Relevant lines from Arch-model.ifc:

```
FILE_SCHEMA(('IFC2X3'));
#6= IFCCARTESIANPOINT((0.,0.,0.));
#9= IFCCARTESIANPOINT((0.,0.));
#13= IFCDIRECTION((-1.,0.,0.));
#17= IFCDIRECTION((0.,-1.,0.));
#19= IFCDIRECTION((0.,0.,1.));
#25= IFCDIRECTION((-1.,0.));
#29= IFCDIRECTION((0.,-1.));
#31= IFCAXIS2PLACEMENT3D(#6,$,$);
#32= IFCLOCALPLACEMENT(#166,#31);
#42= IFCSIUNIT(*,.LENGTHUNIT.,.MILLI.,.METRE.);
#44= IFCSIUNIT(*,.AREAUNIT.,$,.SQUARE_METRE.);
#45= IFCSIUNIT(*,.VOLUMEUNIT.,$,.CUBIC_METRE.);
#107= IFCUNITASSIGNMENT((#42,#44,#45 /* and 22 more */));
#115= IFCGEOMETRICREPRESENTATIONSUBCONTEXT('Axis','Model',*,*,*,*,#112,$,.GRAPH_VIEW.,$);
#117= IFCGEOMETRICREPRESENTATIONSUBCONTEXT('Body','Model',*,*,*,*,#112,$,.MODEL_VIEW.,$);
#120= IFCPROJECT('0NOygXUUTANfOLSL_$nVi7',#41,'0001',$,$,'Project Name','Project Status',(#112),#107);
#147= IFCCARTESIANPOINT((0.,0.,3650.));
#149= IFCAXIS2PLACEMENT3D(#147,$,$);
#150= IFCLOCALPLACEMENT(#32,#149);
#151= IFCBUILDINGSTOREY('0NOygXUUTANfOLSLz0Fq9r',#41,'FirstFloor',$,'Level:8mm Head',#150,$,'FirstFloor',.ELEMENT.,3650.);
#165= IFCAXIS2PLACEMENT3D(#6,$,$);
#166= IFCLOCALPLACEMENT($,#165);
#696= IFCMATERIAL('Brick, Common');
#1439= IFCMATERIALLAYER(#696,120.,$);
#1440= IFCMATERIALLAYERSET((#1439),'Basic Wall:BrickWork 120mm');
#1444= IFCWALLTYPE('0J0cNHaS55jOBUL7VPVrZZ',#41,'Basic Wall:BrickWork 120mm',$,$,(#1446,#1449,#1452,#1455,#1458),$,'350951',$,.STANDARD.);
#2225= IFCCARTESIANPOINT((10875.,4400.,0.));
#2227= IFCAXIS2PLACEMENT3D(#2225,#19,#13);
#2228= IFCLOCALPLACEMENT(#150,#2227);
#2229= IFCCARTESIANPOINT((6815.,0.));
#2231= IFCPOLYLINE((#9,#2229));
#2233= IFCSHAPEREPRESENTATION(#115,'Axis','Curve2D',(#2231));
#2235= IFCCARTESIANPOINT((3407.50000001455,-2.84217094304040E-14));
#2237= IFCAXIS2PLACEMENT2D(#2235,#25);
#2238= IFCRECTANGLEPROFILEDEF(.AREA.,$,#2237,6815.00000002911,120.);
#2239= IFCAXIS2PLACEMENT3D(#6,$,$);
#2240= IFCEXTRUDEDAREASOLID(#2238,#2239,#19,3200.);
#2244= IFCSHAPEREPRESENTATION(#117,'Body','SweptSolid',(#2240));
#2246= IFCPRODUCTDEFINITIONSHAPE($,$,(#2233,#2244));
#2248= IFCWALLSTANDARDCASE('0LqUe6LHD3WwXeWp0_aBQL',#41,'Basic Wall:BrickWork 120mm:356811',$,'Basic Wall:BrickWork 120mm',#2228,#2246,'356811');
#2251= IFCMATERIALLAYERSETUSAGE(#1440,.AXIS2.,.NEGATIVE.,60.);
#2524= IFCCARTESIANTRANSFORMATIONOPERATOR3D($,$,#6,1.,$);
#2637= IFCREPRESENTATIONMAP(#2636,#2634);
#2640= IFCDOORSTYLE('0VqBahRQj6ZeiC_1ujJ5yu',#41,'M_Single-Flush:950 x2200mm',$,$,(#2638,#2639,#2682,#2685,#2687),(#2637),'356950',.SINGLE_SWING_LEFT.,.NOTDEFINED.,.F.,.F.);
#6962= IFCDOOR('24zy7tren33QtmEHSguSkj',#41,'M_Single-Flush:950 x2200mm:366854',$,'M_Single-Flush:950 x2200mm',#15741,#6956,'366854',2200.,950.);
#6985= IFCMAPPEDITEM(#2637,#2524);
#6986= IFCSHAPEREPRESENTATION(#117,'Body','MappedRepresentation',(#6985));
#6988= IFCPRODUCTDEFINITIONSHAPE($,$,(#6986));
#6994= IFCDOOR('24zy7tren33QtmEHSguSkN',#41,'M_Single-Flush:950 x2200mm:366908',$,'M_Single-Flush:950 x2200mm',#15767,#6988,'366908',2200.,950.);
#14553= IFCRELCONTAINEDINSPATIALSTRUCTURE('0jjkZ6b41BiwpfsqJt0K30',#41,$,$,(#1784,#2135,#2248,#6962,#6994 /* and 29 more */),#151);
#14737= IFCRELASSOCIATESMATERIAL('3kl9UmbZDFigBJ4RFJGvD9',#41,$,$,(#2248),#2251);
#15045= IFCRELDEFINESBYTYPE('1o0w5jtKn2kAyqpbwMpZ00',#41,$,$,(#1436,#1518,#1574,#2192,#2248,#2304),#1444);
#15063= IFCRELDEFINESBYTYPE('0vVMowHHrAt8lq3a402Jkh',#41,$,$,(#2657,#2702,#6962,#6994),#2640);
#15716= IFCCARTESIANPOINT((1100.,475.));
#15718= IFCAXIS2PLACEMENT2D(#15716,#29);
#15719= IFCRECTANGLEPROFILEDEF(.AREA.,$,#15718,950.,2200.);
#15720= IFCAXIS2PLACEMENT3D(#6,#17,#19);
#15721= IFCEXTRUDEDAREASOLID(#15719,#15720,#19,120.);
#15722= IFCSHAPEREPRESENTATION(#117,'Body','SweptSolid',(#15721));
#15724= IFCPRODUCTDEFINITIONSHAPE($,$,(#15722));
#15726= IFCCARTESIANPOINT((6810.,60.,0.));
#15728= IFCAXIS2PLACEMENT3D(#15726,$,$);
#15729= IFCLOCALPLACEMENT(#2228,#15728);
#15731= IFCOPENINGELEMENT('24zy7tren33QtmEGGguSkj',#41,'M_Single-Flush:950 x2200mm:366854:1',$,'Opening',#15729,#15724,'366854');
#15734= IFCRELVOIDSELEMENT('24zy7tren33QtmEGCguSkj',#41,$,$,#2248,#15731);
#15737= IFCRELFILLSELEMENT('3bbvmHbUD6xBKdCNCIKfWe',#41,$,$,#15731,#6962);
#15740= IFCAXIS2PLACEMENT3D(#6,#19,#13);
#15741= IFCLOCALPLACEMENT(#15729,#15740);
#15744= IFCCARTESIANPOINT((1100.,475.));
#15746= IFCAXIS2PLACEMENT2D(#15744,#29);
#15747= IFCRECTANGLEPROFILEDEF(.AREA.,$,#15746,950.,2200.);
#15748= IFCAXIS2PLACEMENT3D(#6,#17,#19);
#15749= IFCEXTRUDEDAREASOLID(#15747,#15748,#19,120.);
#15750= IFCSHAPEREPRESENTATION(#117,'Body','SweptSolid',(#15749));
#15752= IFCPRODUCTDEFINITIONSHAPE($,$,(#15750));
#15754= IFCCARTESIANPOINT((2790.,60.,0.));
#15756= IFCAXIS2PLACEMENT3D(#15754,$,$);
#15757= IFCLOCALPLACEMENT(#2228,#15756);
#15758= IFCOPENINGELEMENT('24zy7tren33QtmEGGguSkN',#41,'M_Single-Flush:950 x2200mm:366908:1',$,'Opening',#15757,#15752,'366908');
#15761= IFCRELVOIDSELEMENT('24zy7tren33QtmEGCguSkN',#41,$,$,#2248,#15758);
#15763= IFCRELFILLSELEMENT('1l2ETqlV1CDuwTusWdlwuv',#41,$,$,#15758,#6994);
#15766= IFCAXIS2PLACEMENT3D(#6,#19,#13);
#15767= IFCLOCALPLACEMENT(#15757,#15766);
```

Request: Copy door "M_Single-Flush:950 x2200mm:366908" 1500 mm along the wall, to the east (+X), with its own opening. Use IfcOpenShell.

```python
import ifcopenshell
import ifcopenshell.api.feature
import ifcopenshell.api.geometry
import ifcopenshell.api.root
import ifcopenshell.geom
import ifcopenshell.util.element
import ifcopenshell.util.placement
import ifcopenshell.util.shape
import ifcopenshell.util.unit

model = ifcopenshell.open("Arch-model.ifc")
unit_scale = ifcopenshell.util.unit.calculate_unit_scale(model)
settings = ifcopenshell.geom.settings()


def volume(element):
    """Net volume in cubic metres, openings subtracted."""
    shape = ifcopenshell.geom.create_shape(settings, element)
    return ifcopenshell.util.shape.get_volume(shape.geometry)


def reuse_history(source, copy):
    """copy_class also copies each property set's owner history, people and application; keep the originals."""
    for rel in copy.IsDefinedBy:
        if rel.is_a("IfcRelDefinesByProperties") and (history := rel.RelatingPropertyDefinition.OwnerHistory):
            rel.RelatingPropertyDefinition.OwnerHistory = source.OwnerHistory
            ifcopenshell.util.element.remove_deep2(model, history)


door = model.by_guid("24zy7tren33QtmEHSguSkN")
opening = door.FillsVoids[0].RelatingOpeningElement
wall = opening.VoidsElements[0].RelatingBuildingElement
before = volume(wall)
shift = ifcopenshell.util.placement.get_local_placement(wall.ObjectPlacement)[:3, 0] * -1.5 / unit_scale

# copy_class copies the void relationship, type, container and properties, but no geometry.
new_opening = ifcopenshell.api.root.copy_class(model, product=opening)
new_opening.Representation = ifcopenshell.util.element.copy_deep(
    model, opening.Representation, exclude=["IfcGeometricRepresentationContext", "IfcRepresentationMap"]
)
new_opening.Name = "M_Single-Flush:950 x2200mm"
new_opening.Tag = None
new_door = ifcopenshell.api.root.copy_class(model, product=door)
new_door.Representation = ifcopenshell.util.element.copy_deep(
    model, door.Representation, exclude=["IfcGeometricRepresentationContext", "IfcRepresentationMap"]
)
new_door.Name = "M_Single-Flush:950 x2200mm"
new_door.Tag = None
reuse_history(door, new_door)
fills = ifcopenshell.api.feature.add_filling(model, opening=new_opening, element=new_door)
fills.OwnerHistory = new_door.OwnerHistory  # required in IFC2X3

for old, new in ((opening, new_opening), (door, new_door)):
    matrix = ifcopenshell.util.placement.get_local_placement(old.ObjectPlacement)
    matrix[:3, 3] += shift
    ifcopenshell.api.geometry.edit_object_placement(model, product=new, matrix=matrix, is_si=False)

after = volume(wall)

print(f"wall volume {before:.3f} -> {after:.3f} m3")

model.write("Arch-model_v2.ifc")
```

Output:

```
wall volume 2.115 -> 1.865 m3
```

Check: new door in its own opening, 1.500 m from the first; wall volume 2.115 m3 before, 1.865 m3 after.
